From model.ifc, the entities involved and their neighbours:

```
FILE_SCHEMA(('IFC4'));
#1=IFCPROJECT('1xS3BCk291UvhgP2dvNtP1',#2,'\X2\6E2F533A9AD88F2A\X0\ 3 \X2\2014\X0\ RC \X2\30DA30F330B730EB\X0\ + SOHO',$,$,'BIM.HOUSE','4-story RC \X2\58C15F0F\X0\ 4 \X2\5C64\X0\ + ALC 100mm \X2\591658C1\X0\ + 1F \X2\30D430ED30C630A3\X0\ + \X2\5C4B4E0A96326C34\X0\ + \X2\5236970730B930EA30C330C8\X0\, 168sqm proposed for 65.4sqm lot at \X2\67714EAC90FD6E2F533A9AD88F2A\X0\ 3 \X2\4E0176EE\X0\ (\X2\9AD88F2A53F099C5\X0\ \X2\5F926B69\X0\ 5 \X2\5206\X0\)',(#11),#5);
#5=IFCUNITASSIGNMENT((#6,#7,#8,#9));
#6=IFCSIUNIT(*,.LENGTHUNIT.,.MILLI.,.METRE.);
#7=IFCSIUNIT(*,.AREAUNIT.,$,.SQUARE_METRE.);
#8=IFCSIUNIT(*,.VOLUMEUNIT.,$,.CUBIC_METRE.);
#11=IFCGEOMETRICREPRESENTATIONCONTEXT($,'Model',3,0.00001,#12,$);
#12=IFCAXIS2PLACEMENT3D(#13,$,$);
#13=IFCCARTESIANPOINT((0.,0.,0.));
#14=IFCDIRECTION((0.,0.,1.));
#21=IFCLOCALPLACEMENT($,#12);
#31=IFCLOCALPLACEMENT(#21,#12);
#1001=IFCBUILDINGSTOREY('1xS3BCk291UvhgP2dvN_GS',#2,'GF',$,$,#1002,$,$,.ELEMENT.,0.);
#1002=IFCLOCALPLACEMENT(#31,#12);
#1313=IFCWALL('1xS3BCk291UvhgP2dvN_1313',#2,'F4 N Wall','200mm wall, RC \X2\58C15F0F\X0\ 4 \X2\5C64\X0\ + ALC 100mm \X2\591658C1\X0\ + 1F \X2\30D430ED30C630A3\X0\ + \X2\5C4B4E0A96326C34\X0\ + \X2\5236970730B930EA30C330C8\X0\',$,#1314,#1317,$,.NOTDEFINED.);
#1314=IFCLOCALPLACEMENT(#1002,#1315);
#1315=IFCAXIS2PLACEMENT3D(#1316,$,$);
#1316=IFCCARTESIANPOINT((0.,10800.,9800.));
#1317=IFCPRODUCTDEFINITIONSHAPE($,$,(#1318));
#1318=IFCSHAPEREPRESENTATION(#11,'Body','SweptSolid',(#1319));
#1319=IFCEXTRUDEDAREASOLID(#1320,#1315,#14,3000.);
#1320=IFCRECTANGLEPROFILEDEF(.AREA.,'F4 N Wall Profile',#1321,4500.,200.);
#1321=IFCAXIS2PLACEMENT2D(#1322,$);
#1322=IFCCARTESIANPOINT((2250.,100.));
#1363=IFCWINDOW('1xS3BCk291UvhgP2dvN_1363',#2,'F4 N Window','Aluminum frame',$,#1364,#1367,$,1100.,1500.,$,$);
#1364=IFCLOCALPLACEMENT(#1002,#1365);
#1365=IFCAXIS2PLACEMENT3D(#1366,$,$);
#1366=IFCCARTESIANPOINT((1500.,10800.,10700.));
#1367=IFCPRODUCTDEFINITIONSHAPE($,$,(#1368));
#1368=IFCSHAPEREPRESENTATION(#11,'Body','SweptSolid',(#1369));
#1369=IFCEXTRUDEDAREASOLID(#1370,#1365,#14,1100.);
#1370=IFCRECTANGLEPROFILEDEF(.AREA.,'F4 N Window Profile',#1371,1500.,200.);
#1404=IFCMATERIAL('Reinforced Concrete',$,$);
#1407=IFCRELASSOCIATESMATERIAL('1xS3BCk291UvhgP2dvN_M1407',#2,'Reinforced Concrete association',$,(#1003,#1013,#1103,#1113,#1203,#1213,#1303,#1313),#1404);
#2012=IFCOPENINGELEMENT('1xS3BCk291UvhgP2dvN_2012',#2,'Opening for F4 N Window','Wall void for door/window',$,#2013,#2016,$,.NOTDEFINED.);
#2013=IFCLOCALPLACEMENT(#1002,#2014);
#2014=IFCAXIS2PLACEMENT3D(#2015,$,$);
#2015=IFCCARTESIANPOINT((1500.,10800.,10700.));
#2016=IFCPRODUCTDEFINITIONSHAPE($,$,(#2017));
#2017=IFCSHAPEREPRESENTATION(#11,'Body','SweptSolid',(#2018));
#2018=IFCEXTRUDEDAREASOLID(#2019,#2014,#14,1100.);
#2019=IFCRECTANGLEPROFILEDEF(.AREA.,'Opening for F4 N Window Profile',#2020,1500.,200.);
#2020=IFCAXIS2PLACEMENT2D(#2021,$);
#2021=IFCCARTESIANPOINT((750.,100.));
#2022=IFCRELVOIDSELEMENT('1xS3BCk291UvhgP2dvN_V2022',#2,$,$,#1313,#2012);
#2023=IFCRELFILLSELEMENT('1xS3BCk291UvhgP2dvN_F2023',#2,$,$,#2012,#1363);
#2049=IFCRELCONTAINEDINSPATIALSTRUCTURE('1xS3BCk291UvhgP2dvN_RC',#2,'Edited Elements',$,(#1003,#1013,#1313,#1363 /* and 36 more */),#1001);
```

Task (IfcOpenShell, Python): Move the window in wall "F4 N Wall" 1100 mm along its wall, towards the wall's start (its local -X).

```python
import ifcopenshell
import ifcopenshell.api.geometry
import ifcopenshell.util.placement
import ifcopenshell.util.unit

model = ifcopenshell.open("model.ifc")
unit_scale = ifcopenshell.util.unit.calculate_unit_scale(model)

window = model.by_guid("1xS3BCk291UvhgP2dvN_1363")
opening = window.FillsVoids[0].RelatingOpeningElement
wall = opening.VoidsElements[0].RelatingBuildingElement

wall_matrix = ifcopenshell.util.placement.get_local_placement(wall.ObjectPlacement)
shift = wall_matrix[:3, 0] * -1.1 / unit_scale
before = ifcopenshell.util.placement.get_local_placement(window.ObjectPlacement)[:3, 3].copy()

# The window is not placed relative to its opening, so move both.
for product in (opening, window):
    matrix = ifcopenshell.util.placement.get_local_placement(product.ObjectPlacement)
    matrix[:3, 3] += shift
    ifcopenshell.api.geometry.edit_object_placement(model, product=product, matrix=matrix, is_si=False)

after = ifcopenshell.util.placement.get_local_placement(window.ObjectPlacement)[:3, 3]
print("window moved by", (after - before).round(3) + 0.0)

model.write("model_rev.ifc")
```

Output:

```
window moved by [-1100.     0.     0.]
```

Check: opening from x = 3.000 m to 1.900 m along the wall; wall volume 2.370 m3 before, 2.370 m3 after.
